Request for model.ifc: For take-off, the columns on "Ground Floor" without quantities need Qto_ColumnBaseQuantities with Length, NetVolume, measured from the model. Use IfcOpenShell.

First a look at what the model holds.

```python
import ifcopenshell
import ifcopenshell.util.element
import ifcopenshell.util.unit

model = ifcopenshell.open("model.ifc")
print(model.schema)
for unit_type in ("LENGTHUNIT", "AREAUNIT", "VOLUMEUNIT"):
    print(unit_type, ifcopenshell.util.unit.calculate_unit_scale(model, unit_type))
storey = next(s for s in model.by_type("IfcBuildingStorey") if s.Name == "Ground Floor")
columns = [e for e in ifcopenshell.util.element.get_decomposition(storey) if e.is_a("IfcColumn")]
for e in sorted(columns, key=lambda e: e.id()):
    print(e.id(), e.is_a(), e.Name, list(ifcopenshell.util.element.get_psets(e, qtos_only=True)), sep=" | ")
```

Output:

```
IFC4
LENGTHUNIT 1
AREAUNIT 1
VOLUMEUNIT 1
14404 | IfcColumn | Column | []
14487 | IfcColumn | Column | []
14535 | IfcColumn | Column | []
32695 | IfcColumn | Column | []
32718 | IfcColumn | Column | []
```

```python
import ifcopenshell
import ifcopenshell.api.pset
import ifcopenshell.geom
import ifcopenshell.util.element
import ifcopenshell.util.shape
import ifcopenshell.util.unit

model = ifcopenshell.open("model.ifc")
unit_scale = ifcopenshell.util.unit.calculate_unit_scale(model)
volume_scale = ifcopenshell.util.unit.calculate_unit_scale(model, "VOLUMEUNIT")
settings = ifcopenshell.geom.settings()

storey = next(s for s in model.by_type("IfcBuildingStorey") if s.Name == "Ground Floor")
columns = [e for e in ifcopenshell.util.element.get_decomposition(storey) if e.is_a("IfcColumn")]

for e in sorted(columns, key=lambda e: e.id()):
    if ifcopenshell.util.element.get_psets(e, qtos_only=True, should_inherit=False):
        continue
    # Geometry comes back in metres, in the element's own axes.
    shape = ifcopenshell.geom.create_shape(settings, e)
    values = {
        "Length": ifcopenshell.util.shape.get_z(shape.geometry) / unit_scale,
        "NetVolume": ifcopenshell.util.shape.get_volume(shape.geometry) / volume_scale,
    }
    qto = ifcopenshell.api.pset.add_qto(model, product=e, name="Qto_ColumnBaseQuantities")
    ifcopenshell.api.pset.edit_qto(model, qto=qto, properties=values)
    print(e.id(), {k: round(v, 3) for k, v in values.items()})

model.write("model_edited.ifc")
```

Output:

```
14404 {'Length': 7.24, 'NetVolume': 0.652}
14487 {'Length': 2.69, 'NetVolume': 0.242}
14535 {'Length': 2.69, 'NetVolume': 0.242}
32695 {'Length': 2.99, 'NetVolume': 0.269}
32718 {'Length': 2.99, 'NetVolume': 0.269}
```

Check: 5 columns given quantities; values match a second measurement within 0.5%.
